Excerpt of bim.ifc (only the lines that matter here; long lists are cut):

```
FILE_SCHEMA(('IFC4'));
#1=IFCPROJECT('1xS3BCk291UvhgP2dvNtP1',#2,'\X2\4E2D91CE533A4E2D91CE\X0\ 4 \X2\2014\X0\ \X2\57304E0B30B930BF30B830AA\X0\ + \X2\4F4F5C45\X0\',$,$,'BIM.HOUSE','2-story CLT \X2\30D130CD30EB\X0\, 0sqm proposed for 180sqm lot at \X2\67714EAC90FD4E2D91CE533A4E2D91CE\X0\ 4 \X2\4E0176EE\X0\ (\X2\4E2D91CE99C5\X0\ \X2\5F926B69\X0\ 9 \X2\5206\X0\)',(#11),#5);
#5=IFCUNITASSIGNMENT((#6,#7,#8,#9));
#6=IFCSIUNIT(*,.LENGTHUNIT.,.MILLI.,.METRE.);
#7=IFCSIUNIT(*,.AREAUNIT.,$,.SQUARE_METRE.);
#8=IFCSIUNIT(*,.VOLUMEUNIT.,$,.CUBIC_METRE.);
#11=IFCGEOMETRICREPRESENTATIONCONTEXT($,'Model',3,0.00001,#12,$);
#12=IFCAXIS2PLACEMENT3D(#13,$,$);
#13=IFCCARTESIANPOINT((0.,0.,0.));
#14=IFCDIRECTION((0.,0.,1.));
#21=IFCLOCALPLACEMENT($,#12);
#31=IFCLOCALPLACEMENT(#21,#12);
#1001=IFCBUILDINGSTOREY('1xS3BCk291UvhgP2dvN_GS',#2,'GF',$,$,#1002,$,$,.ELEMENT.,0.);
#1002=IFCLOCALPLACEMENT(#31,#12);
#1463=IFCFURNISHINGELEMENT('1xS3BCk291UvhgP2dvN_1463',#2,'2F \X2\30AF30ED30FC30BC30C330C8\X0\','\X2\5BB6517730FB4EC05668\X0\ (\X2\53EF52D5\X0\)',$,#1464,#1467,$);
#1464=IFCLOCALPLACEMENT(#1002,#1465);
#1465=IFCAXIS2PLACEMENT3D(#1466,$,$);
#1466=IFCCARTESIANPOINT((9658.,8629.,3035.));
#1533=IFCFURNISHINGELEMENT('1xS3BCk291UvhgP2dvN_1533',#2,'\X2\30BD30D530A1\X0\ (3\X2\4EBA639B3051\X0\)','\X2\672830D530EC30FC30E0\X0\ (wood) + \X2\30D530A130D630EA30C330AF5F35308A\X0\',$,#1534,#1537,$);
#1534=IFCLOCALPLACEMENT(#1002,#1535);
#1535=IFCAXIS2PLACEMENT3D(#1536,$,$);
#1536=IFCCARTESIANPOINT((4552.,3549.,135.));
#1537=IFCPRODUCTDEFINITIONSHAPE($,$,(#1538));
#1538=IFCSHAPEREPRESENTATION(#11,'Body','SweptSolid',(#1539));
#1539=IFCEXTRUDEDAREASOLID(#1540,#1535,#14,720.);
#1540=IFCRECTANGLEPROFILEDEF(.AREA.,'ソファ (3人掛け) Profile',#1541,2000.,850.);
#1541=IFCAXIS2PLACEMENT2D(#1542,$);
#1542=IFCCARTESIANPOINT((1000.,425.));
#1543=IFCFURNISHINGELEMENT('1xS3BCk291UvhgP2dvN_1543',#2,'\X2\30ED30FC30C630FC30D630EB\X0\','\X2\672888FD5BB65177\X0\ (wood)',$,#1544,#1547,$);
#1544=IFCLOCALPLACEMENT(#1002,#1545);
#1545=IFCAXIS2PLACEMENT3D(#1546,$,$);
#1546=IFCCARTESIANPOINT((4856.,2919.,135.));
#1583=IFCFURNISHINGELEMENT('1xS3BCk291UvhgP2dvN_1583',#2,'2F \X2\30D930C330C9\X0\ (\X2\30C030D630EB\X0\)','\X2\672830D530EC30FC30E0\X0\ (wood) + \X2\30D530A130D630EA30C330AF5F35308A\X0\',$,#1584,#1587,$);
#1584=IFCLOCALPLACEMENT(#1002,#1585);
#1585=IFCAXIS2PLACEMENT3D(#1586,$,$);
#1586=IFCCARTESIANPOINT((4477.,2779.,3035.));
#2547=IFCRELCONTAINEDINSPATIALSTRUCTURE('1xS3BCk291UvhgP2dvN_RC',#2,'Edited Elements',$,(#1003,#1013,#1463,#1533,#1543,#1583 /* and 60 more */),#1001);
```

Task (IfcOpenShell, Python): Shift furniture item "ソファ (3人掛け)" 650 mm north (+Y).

```python
import ifcopenshell
import ifcopenshell.api.geometry
import ifcopenshell.util.placement

model = ifcopenshell.open("bim.ifc")

item = model.by_guid("1xS3BCk291UvhgP2dvN_1533")
matrix = ifcopenshell.util.placement.get_local_placement(item.ObjectPlacement)
matrix[1, 3] += 650.0
ifcopenshell.api.geometry.edit_object_placement(model, product=item, matrix=matrix, is_si=False)

print(ifcopenshell.util.placement.get_local_placement(item.ObjectPlacement).round(3) + 0.0)

model.write("bim_rev.ifc")
```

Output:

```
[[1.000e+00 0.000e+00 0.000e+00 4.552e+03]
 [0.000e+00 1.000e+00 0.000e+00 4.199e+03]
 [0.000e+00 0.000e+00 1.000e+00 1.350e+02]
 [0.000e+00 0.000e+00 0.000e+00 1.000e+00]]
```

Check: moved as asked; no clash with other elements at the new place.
